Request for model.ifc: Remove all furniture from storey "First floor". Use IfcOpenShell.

First a look at what the model holds.

```python
import ifcopenshell
import ifcopenshell.util.element

model = ifcopenshell.open("model.ifc")
print(model.schema)
storey = next(s for s in model.by_type("IfcBuildingStorey") if s.Name == "First floor")
furniture = [e for e in ifcopenshell.util.element.get_decomposition(storey) if e.is_a("IfcFurnishingElement")]
seen = {}
for e in furniture:
    element_type = ifcopenshell.util.element.get_type(e)
    name = element_type.Name if element_type not in (None, e) else None
    seen[name] = seen.get(name, 0) + 1
for name, count in sorted(seen.items(), key=str):
    print(count, "x", name)
```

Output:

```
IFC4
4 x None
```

```python
import ifcopenshell
import ifcopenshell.api.root
import ifcopenshell.util.element

model = ifcopenshell.open("model.ifc")

storey = next(s for s in model.by_type("IfcBuildingStorey") if s.Name == "First floor")
furniture = [e for e in ifcopenshell.util.element.get_decomposition(storey) if e.is_a("IfcFurnishingElement")]

for e in furniture:
    ifcopenshell.api.root.remove_product(model, product=e)
print(len(furniture), "removed")

model.write("model_updated.ifc")
```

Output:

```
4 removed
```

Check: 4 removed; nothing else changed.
